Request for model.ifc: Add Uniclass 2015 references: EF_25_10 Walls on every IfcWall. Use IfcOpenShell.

First a look at what the model holds.

```python
import ifcopenshell

model = ifcopenshell.open("model.ifc")
print(model.schema)
print("classifications:", [c.Name for c in model.by_type("IfcClassification")])
for ifc_class in ("IfcDoor", "IfcRoof", "IfcStair", "IfcWall", "IfcWindow"):
    print(ifc_class, len(model.by_type(ifc_class)))
```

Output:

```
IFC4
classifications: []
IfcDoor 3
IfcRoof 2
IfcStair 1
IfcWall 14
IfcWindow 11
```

```python
import ifcopenshell
import ifcopenshell.api.classification

model = ifcopenshell.open("model.ifc")

system = ifcopenshell.api.classification.add_classification(model, classification="Uniclass 2015")

codes = {
    "IfcWall": ("EF_25_10", "Walls"),
}
for ifc_class, (code, name) in codes.items():
    products = model.by_type(ifc_class)
    ifcopenshell.api.classification.add_reference(
        model, products=products, classification=system, identification=code, name=name
    )
    print(code, len(products))

model.write("model_updated.ifc")
```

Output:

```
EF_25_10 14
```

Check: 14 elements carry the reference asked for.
